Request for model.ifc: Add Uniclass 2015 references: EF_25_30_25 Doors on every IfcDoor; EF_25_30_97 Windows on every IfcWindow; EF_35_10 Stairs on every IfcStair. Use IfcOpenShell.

First a look at what the model holds.

```python
import ifcopenshell

model = ifcopenshell.open("model.ifc")
print(model.schema)
print("classifications:", [c.Name for c in model.by_type("IfcClassification")])
for ifc_class in ("IfcDoor", "IfcRoof", "IfcStair", "IfcWall", "IfcWindow"):
    print(ifc_class, len(model.by_type(ifc_class)))
```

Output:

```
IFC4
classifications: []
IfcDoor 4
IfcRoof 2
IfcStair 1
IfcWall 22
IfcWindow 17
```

```python
import ifcopenshell
import ifcopenshell.api.classification

model = ifcopenshell.open("model.ifc")

system = ifcopenshell.api.classification.add_classification(model, classification="Uniclass 2015")

codes = {
    "IfcDoor": ("EF_25_30_25", "Doors"),
    "IfcWindow": ("EF_25_30_97", "Windows"),
    "IfcStair": ("EF_35_10", "Stairs"),
}
for ifc_class, (code, name) in codes.items():
    products = model.by_type(ifc_class)
    ifcopenshell.api.classification.add_reference(
        model, products=products, classification=system, identification=code, name=name
    )
    print(code, len(products))

model.write("model_v2.ifc")
```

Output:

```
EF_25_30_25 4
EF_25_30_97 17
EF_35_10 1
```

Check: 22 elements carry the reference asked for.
